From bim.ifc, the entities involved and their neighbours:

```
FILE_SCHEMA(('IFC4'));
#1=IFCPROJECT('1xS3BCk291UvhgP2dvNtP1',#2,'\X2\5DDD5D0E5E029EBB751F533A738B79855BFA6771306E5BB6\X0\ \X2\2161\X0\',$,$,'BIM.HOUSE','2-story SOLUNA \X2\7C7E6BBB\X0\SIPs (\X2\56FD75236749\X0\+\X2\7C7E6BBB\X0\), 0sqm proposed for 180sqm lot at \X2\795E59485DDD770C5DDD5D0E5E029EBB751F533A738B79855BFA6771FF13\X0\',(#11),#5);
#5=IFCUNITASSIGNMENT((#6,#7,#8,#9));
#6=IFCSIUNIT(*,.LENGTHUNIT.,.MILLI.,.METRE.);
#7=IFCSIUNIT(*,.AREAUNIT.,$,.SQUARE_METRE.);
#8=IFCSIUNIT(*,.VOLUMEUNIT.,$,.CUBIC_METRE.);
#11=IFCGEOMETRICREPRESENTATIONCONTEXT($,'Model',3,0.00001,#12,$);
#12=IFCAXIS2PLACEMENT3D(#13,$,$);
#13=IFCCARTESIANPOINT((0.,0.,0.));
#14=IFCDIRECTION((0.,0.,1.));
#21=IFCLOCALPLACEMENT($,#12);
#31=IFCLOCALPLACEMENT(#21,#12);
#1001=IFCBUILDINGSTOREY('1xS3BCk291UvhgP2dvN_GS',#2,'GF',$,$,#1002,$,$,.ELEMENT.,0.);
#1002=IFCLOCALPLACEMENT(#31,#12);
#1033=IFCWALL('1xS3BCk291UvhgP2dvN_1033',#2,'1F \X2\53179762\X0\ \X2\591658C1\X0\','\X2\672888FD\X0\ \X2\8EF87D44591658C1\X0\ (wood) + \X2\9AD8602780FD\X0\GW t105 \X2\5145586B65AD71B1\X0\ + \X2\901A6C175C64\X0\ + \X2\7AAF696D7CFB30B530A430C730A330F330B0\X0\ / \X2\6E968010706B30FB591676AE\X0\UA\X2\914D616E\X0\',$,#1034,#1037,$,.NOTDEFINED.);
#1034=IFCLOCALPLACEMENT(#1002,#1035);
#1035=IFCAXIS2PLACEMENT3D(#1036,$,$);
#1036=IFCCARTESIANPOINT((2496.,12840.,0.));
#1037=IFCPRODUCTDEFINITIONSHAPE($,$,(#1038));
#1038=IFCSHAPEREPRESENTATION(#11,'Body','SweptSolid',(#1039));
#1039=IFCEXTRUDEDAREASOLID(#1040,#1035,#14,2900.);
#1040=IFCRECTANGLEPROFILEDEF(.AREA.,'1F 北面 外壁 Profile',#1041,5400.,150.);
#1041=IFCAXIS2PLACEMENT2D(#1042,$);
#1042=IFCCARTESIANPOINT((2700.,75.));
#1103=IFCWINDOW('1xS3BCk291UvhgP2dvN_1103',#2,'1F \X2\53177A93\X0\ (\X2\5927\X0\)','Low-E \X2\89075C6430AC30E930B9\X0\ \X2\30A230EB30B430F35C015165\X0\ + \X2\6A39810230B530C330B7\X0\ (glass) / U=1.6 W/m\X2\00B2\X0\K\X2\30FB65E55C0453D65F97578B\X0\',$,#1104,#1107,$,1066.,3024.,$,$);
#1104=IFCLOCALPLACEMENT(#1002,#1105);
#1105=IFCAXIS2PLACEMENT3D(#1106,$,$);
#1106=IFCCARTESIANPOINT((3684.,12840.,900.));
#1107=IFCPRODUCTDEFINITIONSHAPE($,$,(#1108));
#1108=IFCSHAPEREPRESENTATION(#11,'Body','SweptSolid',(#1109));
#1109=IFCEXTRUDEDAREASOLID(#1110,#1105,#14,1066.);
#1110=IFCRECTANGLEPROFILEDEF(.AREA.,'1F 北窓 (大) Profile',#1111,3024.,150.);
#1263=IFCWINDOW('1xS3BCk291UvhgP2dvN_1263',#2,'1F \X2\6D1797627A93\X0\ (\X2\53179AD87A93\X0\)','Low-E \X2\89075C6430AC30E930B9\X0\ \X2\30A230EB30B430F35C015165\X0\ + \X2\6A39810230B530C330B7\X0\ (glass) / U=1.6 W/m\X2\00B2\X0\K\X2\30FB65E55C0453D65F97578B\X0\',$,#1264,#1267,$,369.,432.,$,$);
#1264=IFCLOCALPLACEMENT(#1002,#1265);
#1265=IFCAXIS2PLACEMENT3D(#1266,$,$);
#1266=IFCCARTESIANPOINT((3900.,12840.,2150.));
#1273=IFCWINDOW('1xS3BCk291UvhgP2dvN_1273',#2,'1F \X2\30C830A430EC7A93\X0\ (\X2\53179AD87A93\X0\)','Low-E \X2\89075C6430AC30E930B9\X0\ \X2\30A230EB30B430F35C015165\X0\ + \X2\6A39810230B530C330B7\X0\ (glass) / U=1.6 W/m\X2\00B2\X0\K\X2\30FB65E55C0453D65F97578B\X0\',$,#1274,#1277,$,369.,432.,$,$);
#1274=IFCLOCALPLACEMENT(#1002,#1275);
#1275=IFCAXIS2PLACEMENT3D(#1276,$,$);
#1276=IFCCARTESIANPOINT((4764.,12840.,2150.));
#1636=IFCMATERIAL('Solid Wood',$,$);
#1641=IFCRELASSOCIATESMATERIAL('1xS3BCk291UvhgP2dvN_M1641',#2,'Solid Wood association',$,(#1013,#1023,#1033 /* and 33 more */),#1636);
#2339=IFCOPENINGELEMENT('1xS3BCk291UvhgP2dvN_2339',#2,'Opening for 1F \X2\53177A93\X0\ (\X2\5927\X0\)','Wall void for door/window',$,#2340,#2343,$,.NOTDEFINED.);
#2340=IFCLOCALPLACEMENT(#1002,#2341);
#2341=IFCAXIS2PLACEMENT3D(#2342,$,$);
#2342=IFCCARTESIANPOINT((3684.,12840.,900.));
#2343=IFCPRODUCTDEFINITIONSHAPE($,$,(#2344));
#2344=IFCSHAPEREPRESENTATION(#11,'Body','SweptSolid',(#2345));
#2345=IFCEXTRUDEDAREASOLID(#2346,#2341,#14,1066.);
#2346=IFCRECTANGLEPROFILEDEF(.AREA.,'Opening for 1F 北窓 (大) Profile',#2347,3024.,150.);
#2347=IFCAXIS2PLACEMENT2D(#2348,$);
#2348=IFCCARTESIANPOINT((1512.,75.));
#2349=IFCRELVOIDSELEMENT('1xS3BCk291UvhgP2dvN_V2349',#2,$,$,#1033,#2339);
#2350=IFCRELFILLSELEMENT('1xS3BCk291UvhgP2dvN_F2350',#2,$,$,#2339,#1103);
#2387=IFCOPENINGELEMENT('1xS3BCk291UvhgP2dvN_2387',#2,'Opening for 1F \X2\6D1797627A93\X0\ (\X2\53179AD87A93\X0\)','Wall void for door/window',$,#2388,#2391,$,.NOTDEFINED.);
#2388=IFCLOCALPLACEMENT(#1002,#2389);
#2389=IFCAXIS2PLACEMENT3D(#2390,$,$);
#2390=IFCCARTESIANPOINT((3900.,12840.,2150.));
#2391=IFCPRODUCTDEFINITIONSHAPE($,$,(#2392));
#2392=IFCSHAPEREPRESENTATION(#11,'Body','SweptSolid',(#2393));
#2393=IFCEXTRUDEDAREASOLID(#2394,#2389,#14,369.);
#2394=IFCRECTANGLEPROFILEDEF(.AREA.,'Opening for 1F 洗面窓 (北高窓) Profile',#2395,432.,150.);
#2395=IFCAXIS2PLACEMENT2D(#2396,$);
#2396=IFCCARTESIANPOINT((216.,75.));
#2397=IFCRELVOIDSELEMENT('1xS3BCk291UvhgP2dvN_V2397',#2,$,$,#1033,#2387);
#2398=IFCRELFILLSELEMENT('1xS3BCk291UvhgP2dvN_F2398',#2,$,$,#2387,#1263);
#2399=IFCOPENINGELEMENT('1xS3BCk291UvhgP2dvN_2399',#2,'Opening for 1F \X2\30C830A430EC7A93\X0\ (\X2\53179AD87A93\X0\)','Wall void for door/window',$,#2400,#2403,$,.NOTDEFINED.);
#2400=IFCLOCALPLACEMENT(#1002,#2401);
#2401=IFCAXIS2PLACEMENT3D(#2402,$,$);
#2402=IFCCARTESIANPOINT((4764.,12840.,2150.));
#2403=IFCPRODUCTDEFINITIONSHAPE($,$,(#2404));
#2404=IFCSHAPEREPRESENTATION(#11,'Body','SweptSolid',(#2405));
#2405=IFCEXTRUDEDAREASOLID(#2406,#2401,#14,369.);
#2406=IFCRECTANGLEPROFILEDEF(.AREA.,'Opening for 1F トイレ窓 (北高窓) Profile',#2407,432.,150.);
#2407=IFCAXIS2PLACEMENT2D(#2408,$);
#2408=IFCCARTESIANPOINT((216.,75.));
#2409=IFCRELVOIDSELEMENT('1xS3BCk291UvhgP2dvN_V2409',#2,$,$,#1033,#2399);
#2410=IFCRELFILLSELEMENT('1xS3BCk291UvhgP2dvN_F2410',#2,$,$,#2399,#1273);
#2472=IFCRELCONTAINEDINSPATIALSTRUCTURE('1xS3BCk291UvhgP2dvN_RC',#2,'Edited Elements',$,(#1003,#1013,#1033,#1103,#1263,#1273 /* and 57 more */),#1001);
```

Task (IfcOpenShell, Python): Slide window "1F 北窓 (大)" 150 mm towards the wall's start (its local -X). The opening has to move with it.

```python
import ifcopenshell
import ifcopenshell.api.geometry
import ifcopenshell.util.placement
import ifcopenshell.util.unit

model = ifcopenshell.open("bim.ifc")
unit_scale = ifcopenshell.util.unit.calculate_unit_scale(model)

window = model.by_guid("1xS3BCk291UvhgP2dvN_1103")
opening = window.FillsVoids[0].RelatingOpeningElement
wall = opening.VoidsElements[0].RelatingBuildingElement

wall_matrix = ifcopenshell.util.placement.get_local_placement(wall.ObjectPlacement)
shift = wall_matrix[:3, 0] * -0.15 / unit_scale
before = ifcopenshell.util.placement.get_local_placement(window.ObjectPlacement)[:3, 3].copy()

# The window is not placed relative to its opening, so move both.
for product in (opening, window):
    matrix = ifcopenshell.util.placement.get_local_placement(product.ObjectPlacement)
    matrix[:3, 3] += shift
    ifcopenshell.api.geometry.edit_object_placement(model, product=product, matrix=matrix, is_si=False)

after = ifcopenshell.util.placement.get_local_placement(window.ObjectPlacement)[:3, 3]
print("window moved by", (after - before).round(3) + 0.0)

model.write("bim_edited.ifc")
```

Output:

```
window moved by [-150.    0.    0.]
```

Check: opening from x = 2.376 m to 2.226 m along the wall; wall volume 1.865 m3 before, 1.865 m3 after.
